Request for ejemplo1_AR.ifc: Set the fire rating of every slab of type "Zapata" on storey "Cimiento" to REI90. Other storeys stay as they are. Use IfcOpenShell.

First a look at what the model holds.

```python
import ifcopenshell
import ifcopenshell.util.element

model = ifcopenshell.open("ejemplo1_AR.ifc")
print(model.schema)
storey = next(s for s in model.by_type("IfcBuildingStorey") if s.Name == "Cimiento")
slabs = [e for e in ifcopenshell.util.element.get_decomposition(storey) if e.is_a("IfcSlab")]
seen = {}
for e in slabs:
    element_type = ifcopenshell.util.element.get_type(e)
    key = (element_type.Name if element_type != e and element_type else None, ifcopenshell.util.element.get_pset(e, "Pset_SlabCommon", "FireRating"))
    seen[key] = seen.get(key, 0) + 1
for (name, value), count in sorted(seen.items(), key=str):
    print(count, "x", name, "|", value)
```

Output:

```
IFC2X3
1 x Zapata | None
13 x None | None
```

```python
import ifcopenshell
import ifcopenshell.api.pset
import ifcopenshell.util.element

model = ifcopenshell.open("ejemplo1_AR.ifc")

storey = next(s for s in model.by_type("IfcBuildingStorey") if s.Name == "Cimiento")
slabs = [e for e in ifcopenshell.util.element.get_decomposition(storey) if e.is_a("IfcSlab")]

count = 0
for e in slabs:
    element_type = ifcopenshell.util.element.get_type(e)
    if element_type in (None, e) or element_type.Name != "Zapata":
        continue
    # add_pset returns the element's existing set when there is one.
    pset = ifcopenshell.api.pset.add_pset(model, product=e, name="Pset_SlabCommon")
    ifcopenshell.api.pset.edit_pset(model, pset=pset, properties={"FireRating": "REI90"})
    count += 1

print(count, "slabs updated")

model.write("ejemplo1_AR_rev.ifc")
```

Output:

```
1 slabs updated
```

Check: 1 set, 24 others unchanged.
